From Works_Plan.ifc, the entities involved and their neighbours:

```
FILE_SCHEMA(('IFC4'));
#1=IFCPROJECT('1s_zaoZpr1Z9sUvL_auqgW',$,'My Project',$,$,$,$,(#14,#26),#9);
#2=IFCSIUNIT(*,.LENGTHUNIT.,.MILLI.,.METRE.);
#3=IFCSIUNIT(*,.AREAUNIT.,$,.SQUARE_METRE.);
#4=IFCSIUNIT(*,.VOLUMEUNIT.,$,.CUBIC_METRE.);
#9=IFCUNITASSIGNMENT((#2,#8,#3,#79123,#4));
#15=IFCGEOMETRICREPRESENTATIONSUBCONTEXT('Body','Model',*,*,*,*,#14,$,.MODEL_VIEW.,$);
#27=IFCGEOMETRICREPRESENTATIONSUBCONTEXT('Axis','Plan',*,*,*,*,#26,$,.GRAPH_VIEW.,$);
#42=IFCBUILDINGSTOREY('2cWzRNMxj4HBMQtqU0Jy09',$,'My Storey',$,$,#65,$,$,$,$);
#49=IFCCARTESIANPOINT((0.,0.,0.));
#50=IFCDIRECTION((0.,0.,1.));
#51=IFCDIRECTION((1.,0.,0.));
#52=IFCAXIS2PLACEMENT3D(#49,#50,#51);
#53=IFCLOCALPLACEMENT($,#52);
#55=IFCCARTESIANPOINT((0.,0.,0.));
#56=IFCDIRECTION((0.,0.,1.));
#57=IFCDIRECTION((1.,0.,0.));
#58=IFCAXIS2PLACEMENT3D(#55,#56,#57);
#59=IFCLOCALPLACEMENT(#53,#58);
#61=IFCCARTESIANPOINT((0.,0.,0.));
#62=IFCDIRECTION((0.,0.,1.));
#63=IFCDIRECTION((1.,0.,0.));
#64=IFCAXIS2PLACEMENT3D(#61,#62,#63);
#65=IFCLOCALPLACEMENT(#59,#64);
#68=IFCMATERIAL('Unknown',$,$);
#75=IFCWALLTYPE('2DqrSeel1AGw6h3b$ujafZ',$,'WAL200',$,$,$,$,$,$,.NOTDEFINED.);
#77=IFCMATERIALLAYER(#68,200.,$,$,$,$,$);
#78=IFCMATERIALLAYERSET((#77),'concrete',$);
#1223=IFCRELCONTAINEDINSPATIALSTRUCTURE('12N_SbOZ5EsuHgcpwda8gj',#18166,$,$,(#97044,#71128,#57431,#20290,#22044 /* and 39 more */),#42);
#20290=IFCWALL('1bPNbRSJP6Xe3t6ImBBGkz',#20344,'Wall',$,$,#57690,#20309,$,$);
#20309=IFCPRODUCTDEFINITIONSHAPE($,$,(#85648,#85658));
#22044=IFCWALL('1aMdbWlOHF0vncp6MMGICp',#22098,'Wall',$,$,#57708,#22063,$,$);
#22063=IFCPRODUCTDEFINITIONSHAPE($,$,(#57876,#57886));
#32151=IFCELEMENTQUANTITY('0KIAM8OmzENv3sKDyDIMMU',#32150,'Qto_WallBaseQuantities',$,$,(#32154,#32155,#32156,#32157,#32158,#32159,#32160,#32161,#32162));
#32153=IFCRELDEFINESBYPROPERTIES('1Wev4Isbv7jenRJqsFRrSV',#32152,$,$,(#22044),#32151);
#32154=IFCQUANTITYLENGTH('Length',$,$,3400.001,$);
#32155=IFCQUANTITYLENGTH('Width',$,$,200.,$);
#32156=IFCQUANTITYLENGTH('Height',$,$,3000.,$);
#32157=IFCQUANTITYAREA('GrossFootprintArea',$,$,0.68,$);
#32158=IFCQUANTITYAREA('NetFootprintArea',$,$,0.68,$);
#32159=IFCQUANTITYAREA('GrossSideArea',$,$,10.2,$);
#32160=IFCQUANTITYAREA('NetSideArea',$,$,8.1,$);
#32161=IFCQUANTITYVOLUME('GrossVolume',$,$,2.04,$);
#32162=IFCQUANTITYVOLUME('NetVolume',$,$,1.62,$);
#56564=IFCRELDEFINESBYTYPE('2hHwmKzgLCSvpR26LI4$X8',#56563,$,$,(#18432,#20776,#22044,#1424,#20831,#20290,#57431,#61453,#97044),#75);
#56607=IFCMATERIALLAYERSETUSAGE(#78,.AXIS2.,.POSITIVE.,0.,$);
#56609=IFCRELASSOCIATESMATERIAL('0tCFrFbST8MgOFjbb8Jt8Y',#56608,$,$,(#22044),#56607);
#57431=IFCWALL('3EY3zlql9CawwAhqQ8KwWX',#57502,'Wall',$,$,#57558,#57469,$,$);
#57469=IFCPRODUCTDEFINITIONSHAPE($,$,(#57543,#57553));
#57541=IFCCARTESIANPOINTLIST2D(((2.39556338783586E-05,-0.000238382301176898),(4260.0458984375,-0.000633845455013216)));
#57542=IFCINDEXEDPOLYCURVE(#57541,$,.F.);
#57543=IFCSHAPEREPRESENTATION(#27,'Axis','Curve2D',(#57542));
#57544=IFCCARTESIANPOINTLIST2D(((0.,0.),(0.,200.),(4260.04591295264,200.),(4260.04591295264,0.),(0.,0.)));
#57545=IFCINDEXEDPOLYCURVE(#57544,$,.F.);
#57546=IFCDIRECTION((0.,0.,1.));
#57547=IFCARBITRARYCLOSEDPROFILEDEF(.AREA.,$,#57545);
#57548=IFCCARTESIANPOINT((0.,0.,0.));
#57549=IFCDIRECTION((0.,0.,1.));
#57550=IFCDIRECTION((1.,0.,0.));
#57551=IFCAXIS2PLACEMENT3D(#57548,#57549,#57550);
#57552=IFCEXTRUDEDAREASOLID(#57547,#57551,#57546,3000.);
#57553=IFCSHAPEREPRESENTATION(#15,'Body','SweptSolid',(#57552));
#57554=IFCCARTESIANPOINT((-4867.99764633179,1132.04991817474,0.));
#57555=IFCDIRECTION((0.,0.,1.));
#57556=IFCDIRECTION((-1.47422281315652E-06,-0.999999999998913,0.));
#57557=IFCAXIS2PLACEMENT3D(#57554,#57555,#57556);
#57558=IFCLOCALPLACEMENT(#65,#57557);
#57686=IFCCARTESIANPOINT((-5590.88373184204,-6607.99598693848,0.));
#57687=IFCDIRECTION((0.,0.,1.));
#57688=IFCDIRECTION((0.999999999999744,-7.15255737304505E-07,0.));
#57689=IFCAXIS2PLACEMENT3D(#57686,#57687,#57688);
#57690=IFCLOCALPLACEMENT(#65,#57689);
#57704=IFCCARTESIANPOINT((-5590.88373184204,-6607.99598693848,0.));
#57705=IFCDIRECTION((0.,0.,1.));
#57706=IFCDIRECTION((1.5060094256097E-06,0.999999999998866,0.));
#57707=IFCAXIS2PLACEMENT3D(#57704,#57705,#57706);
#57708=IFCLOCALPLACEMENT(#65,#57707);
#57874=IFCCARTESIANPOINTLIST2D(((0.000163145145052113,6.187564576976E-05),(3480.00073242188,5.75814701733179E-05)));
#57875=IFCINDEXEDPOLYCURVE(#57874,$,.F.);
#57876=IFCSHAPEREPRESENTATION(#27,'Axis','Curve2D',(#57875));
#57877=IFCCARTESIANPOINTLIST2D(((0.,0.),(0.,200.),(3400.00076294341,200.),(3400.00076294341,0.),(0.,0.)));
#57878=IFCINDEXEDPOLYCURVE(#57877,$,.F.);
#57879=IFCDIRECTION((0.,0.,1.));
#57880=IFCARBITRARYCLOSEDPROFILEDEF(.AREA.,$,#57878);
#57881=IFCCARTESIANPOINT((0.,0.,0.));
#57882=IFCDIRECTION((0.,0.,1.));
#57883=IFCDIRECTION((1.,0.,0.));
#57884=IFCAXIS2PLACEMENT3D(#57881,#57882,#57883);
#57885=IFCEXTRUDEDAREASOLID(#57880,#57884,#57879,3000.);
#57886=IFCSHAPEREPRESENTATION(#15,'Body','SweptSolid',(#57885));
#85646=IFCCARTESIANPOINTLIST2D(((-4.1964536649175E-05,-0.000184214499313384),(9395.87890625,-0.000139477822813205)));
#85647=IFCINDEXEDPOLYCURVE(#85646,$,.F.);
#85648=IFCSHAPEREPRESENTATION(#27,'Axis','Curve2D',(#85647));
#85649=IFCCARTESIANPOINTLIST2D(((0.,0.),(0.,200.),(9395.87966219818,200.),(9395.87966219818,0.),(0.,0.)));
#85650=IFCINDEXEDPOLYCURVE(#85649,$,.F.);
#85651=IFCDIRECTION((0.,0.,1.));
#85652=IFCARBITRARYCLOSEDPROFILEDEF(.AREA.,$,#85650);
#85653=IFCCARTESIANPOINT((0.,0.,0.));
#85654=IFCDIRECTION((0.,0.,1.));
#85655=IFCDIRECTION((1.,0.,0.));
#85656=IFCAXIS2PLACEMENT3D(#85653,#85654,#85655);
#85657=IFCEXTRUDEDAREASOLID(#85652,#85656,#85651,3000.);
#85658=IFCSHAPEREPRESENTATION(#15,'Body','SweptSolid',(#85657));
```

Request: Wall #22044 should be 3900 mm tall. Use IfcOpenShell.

```python
import ifcopenshell
import ifcopenshell.api.pset
import ifcopenshell.geom
import ifcopenshell.util.element
import ifcopenshell.util.representation
import ifcopenshell.util.shape
import ifcopenshell.util.unit

model = ifcopenshell.open("Works_Plan.ifc")
unit_scale = ifcopenshell.util.unit.calculate_unit_scale(model)
area_scale = ifcopenshell.util.unit.calculate_unit_scale(model, "AREAUNIT")
volume_scale = ifcopenshell.util.unit.calculate_unit_scale(model, "VOLUMEUNIT")
settings = ifcopenshell.geom.settings()


def volume(element):
    """Net volume in cubic metres, openings subtracted."""
    shape = ifcopenshell.geom.create_shape(settings, element)
    return ifcopenshell.util.shape.get_volume(shape.geometry)


wall = model.by_id(22044)
before = volume(wall)

body = ifcopenshell.util.representation.get_representation(wall, "Model", "Body")
solid = body.Items[0]
old_height = solid.Depth
solid.Depth = 3.9 / unit_scale
after = volume(wall)
thickness = 0.2  # wall thickness in metres

# Update the stored height, areas and volumes.
qto = model.by_id(ifcopenshell.util.element.get_pset(wall, "Qto_WallBaseQuantities", should_inherit=False)["id"])
ifcopenshell.api.pset.edit_qto(model, qto=qto, properties={
    "Height": solid.Depth,
    "GrossSideArea": ifcopenshell.util.element.get_pset(wall, "Qto_WallBaseQuantities", "GrossSideArea") * solid.Depth / old_height,
    "NetSideArea": after / thickness / area_scale,
    "GrossVolume": ifcopenshell.util.element.get_pset(wall, "Qto_WallBaseQuantities", "GrossVolume") * solid.Depth / old_height,
    "NetVolume": after / volume_scale,
})

print(f"height {old_height:g} -> {solid.Depth:g}, volume {before:.3f} -> {after:.3f} m3")

model.write("Works_Plan_edited.ifc")
```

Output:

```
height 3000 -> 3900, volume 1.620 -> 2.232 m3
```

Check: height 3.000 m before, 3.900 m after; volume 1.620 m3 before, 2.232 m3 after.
